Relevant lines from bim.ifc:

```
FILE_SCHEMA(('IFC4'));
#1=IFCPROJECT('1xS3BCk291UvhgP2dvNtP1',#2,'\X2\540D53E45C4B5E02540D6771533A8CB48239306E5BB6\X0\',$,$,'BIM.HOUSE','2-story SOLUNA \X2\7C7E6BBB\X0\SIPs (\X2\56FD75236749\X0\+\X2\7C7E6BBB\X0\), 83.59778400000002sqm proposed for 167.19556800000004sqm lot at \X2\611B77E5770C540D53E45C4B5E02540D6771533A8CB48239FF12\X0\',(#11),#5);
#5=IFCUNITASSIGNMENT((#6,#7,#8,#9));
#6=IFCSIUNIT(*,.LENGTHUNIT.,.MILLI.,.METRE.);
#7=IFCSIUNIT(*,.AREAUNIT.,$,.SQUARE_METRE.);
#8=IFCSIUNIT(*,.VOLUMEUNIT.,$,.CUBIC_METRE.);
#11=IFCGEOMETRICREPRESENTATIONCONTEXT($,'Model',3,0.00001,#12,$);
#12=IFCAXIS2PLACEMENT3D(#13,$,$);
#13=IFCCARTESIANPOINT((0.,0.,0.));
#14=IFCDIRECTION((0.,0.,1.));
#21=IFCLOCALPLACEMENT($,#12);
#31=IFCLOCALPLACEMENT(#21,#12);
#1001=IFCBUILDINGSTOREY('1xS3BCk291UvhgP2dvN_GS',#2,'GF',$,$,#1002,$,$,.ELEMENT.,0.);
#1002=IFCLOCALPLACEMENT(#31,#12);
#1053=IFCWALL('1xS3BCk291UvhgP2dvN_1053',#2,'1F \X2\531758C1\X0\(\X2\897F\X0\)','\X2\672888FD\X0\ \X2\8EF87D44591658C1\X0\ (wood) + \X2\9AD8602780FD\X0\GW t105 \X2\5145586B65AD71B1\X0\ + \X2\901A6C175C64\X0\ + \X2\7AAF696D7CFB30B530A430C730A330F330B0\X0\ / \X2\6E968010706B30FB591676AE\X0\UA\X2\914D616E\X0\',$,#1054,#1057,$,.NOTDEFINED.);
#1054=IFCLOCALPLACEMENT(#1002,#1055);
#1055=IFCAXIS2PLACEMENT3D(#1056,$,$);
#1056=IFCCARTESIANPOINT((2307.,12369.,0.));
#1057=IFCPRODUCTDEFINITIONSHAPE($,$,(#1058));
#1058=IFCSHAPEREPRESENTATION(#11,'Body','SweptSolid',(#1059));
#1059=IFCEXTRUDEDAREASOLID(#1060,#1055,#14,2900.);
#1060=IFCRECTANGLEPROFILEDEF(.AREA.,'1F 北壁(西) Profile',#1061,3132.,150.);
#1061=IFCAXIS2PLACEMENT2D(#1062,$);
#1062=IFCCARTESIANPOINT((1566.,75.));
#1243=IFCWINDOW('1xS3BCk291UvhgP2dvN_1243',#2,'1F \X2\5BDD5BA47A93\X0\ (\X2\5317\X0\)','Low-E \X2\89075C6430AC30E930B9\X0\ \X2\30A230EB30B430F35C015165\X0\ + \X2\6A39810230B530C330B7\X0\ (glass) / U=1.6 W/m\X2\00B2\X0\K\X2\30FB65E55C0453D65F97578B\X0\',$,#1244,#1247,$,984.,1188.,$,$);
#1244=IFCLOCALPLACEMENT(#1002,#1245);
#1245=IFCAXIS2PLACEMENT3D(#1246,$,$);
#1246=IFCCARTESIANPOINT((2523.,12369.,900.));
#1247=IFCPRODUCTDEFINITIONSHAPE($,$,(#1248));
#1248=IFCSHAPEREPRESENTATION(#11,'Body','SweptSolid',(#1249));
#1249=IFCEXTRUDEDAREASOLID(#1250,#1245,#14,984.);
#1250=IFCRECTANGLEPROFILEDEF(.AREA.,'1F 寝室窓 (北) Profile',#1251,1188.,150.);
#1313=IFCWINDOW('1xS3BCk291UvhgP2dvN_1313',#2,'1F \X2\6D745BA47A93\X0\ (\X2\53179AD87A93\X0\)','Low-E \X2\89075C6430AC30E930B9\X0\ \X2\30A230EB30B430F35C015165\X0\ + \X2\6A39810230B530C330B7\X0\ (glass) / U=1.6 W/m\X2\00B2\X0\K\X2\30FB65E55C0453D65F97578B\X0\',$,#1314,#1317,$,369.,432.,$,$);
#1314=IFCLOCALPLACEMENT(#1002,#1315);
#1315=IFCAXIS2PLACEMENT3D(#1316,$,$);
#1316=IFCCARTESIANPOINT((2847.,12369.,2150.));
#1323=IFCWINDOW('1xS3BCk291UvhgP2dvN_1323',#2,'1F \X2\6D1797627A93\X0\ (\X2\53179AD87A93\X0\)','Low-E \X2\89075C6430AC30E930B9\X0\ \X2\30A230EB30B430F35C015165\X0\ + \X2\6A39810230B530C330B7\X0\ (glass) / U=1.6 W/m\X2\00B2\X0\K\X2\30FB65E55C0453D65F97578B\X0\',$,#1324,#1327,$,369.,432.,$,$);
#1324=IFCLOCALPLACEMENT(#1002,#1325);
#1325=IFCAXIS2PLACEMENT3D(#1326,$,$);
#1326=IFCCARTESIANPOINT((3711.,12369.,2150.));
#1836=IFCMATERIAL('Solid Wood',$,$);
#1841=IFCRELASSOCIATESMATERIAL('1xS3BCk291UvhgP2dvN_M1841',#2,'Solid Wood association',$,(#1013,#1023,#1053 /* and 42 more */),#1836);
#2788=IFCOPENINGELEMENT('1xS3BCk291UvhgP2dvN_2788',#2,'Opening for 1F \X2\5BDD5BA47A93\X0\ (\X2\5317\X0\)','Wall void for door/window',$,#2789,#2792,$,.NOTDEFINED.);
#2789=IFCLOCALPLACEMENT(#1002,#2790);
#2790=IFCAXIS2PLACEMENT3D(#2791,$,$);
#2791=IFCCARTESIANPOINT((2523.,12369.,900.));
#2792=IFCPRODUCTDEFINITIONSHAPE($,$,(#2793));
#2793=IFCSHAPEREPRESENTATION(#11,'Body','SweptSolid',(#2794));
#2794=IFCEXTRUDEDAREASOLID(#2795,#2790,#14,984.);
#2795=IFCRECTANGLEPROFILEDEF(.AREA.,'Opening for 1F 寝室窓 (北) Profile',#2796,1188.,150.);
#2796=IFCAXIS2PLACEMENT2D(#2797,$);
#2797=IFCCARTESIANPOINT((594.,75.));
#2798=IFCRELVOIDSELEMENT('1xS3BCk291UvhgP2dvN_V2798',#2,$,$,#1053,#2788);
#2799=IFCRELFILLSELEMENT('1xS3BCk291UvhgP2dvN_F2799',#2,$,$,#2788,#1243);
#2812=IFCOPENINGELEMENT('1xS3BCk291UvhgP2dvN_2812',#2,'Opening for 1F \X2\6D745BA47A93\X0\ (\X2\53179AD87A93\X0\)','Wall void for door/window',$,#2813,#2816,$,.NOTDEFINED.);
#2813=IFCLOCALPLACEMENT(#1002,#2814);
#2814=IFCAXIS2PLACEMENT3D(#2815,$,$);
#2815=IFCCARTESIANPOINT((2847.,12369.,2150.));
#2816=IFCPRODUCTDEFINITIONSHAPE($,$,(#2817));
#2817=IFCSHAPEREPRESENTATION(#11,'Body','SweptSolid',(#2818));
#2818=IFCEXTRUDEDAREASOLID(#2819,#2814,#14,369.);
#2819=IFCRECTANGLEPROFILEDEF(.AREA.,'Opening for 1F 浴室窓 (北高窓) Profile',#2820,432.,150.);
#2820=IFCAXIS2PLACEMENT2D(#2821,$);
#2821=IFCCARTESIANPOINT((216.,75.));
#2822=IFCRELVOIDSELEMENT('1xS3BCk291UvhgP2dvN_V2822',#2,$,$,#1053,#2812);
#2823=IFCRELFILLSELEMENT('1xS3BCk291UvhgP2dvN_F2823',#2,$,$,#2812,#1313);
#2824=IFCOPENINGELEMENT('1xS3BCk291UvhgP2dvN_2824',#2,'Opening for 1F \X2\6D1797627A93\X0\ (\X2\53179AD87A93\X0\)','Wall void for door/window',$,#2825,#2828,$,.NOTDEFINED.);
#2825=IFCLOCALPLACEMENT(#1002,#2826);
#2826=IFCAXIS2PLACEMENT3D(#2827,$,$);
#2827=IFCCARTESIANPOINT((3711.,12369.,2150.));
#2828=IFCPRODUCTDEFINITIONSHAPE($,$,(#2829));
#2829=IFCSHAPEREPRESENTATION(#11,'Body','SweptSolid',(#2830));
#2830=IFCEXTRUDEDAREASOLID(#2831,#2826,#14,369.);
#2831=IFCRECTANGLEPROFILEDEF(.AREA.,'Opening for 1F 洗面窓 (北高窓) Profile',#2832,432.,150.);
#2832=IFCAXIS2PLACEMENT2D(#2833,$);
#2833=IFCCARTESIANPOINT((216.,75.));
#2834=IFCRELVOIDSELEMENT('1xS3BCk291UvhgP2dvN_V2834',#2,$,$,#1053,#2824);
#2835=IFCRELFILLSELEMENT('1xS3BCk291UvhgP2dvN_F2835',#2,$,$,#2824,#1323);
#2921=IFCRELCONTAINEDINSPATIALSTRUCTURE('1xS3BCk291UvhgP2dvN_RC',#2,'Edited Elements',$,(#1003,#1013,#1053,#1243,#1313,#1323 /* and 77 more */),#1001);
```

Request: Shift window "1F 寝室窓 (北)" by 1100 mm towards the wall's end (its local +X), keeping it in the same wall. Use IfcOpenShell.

```python
import ifcopenshell
import ifcopenshell.api.geometry
import ifcopenshell.util.placement

model = ifcopenshell.open("bim.ifc")

window = model.by_guid("1xS3BCk291UvhgP2dvN_1243")
opening = window.FillsVoids[0].RelatingOpeningElement
wall = opening.VoidsElements[0].RelatingBuildingElement

wall_matrix = ifcopenshell.util.placement.get_local_placement(wall.ObjectPlacement)
shift = wall_matrix[:3, 0] * 1100.0
before = ifcopenshell.util.placement.get_local_placement(window.ObjectPlacement)[:3, 3].copy()

# The window is not placed relative to its opening, so move both.
for product in (opening, window):
    matrix = ifcopenshell.util.placement.get_local_placement(product.ObjectPlacement)
    matrix[:3, 3] += shift
    ifcopenshell.api.geometry.edit_object_placement(model, product=product, matrix=matrix, is_si=False)

after = ifcopenshell.util.placement.get_local_placement(window.ObjectPlacement)[:3, 3]
print("window moved by", (after - before).round(3) + 0.0)

model.write("bim_rev.ifc")
```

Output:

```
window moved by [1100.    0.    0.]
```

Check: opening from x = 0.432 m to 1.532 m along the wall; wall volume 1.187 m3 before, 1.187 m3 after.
